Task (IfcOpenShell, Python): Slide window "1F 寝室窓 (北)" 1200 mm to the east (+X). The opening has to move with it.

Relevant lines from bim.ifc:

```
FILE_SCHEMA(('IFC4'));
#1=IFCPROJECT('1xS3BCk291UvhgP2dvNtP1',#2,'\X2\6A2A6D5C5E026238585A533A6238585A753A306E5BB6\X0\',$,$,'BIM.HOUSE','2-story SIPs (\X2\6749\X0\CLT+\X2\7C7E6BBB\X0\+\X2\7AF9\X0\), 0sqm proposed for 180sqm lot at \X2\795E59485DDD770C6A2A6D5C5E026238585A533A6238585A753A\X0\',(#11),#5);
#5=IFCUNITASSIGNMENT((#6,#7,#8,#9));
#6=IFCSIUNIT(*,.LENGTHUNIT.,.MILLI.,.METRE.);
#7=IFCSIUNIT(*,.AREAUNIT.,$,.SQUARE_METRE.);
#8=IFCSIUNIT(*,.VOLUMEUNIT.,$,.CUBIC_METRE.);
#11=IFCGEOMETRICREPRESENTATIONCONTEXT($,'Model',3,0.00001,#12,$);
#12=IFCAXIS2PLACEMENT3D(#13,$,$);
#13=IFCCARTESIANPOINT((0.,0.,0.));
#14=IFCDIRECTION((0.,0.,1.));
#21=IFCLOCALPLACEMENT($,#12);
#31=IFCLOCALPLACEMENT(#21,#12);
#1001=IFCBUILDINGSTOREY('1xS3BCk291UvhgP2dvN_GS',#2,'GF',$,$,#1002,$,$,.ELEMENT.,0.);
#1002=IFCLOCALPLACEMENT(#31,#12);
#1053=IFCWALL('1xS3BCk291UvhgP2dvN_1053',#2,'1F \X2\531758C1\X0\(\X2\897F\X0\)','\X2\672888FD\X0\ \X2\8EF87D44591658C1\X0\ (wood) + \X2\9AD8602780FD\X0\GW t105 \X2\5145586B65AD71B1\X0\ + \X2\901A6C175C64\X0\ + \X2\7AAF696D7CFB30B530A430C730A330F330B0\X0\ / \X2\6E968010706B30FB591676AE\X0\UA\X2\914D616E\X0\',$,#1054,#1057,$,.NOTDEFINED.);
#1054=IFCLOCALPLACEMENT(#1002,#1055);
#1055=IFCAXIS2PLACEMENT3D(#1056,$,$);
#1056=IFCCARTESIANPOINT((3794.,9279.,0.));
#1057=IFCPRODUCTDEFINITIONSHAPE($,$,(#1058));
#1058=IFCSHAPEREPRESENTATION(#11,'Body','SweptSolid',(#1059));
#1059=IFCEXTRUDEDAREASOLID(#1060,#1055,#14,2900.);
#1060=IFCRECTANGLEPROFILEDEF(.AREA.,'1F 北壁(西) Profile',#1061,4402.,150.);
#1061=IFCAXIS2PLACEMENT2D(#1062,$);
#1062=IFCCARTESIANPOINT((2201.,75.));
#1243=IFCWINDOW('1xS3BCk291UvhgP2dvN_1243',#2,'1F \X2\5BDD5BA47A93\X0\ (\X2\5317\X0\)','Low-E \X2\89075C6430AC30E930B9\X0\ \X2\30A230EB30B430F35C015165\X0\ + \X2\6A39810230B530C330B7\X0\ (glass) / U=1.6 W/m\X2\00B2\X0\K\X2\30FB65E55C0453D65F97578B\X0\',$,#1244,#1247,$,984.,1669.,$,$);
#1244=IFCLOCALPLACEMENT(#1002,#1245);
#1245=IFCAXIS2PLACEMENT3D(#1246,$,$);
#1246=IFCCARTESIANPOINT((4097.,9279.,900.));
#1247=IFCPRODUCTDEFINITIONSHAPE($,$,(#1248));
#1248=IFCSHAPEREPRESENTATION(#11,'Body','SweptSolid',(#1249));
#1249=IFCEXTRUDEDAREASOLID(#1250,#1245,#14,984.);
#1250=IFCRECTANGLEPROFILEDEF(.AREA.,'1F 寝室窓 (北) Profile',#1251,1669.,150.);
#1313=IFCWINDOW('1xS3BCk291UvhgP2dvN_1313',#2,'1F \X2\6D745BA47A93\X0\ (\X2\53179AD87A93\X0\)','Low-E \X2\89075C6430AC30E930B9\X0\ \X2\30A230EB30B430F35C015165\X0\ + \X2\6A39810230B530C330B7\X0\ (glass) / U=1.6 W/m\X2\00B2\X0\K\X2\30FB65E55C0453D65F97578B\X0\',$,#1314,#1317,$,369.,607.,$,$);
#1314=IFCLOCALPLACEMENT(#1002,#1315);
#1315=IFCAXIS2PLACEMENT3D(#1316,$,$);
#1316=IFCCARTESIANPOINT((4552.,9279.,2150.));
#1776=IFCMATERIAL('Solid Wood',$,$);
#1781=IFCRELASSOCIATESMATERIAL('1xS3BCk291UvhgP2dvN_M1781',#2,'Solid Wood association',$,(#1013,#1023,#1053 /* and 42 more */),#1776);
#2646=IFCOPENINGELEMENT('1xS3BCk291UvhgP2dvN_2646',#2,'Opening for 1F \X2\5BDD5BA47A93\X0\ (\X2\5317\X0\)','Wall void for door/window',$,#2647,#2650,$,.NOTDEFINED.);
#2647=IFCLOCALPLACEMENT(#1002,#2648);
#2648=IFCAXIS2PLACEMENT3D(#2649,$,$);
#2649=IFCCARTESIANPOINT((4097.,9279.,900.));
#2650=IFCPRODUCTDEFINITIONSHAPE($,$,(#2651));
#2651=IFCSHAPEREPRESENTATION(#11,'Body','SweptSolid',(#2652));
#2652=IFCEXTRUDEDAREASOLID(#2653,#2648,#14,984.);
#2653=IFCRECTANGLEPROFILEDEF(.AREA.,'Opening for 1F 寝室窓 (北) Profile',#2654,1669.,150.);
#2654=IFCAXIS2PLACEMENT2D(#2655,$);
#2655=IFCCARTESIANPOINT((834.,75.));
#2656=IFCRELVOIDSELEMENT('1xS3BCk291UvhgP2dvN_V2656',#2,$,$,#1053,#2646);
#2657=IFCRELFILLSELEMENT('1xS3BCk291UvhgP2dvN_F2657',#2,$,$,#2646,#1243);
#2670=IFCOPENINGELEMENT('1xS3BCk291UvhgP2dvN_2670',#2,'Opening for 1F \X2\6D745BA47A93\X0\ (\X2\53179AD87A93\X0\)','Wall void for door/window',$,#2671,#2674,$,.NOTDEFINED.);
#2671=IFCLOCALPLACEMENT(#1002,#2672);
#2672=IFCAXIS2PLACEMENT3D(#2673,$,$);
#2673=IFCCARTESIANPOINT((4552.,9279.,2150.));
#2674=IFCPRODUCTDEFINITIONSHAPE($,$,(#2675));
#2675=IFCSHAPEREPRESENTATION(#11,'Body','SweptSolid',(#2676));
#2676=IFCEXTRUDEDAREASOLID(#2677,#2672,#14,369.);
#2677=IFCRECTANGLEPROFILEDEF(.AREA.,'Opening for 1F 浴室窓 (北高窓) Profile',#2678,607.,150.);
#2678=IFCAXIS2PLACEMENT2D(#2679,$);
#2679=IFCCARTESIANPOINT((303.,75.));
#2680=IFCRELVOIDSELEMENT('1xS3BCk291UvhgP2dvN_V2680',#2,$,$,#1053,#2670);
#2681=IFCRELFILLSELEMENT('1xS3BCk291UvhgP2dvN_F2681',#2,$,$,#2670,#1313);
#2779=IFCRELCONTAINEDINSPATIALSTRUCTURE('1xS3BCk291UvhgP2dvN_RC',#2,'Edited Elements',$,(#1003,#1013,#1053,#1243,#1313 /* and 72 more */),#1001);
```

```python
import ifcopenshell
import ifcopenshell.api.geometry
import ifcopenshell.util.placement
import ifcopenshell.util.unit

model = ifcopenshell.open("bim.ifc")
unit_scale = ifcopenshell.util.unit.calculate_unit_scale(model)

window = model.by_guid("1xS3BCk291UvhgP2dvN_1243")
opening = window.FillsVoids[0].RelatingOpeningElement
wall = opening.VoidsElements[0].RelatingBuildingElement

wall_matrix = ifcopenshell.util.placement.get_local_placement(wall.ObjectPlacement)
shift = wall_matrix[:3, 0] * 1.2 / unit_scale
before = ifcopenshell.util.placement.get_local_placement(window.ObjectPlacement)[:3, 3].copy()

# The window is not placed relative to its opening, so move both.
for product in (opening, window):
    matrix = ifcopenshell.util.placement.get_local_placement(product.ObjectPlacement)
    matrix[:3, 3] += shift
    ifcopenshell.api.geometry.edit_object_placement(model, product=product, matrix=matrix, is_si=False)

after = ifcopenshell.util.placement.get_local_placement(window.ObjectPlacement)[:3, 3]
print("window moved by", (after - before).round(3) + 0.0)

model.write("bim_updated.ifc")
```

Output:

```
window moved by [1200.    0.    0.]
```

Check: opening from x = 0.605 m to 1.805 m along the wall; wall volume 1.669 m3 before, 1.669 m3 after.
